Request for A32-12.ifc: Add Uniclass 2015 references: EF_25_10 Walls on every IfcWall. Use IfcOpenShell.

First a look at what the model holds.

```python
import ifcopenshell

model = ifcopenshell.open("A32-12.ifc")
print(model.schema)
print("classifications:", [c.Name for c in model.by_type("IfcClassification")])
for ifc_class in ("IfcDoor", "IfcRoof", "IfcStair", "IfcWall", "IfcWindow"):
    print(ifc_class, len(model.by_type(ifc_class)))
```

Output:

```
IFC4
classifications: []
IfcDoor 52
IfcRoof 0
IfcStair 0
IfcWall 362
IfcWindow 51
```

```python
import ifcopenshell
import ifcopenshell.api.classification

model = ifcopenshell.open("A32-12.ifc")

system = ifcopenshell.api.classification.add_classification(model, classification="Uniclass 2015")

codes = {
    "IfcWall": ("EF_25_10", "Walls"),
}
for ifc_class, (code, name) in codes.items():
    products = model.by_type(ifc_class)
    ifcopenshell.api.classification.add_reference(
        model, products=products, classification=system, identification=code, name=name
    )
    print(code, len(products))

model.write("A32-12_updated.ifc")
```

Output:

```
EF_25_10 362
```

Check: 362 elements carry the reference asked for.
